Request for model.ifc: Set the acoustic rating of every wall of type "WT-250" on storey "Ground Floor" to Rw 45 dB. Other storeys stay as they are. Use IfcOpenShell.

First a look at what the model holds.

```python
import ifcopenshell
import ifcopenshell.util.element

model = ifcopenshell.open("model.ifc")
print(model.schema)
storey = next(s for s in model.by_type("IfcBuildingStorey") if s.Name == "Ground Floor")
walls = [e for e in ifcopenshell.util.element.get_decomposition(storey) if e.is_a("IfcWall")]
seen = {}
for e in walls:
    element_type = ifcopenshell.util.element.get_type(e)
    key = (element_type.Name if element_type != e and element_type else None, ifcopenshell.util.element.get_pset(e, "Pset_WallCommon", "AcousticRating"))
    seen[key] = seen.get(key, 0) + 1
for (name, value), count in sorted(seen.items(), key=str):
    print(count, "x", name, "|", value)
```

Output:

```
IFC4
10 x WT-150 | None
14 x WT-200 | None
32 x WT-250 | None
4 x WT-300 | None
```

```python
import ifcopenshell
import ifcopenshell.api.pset
import ifcopenshell.util.element

model = ifcopenshell.open("model.ifc")

storey = next(s for s in model.by_type("IfcBuildingStorey") if s.Name == "Ground Floor")
walls = [e for e in ifcopenshell.util.element.get_decomposition(storey) if e.is_a("IfcWall")]

count = 0
for e in walls:
    element_type = ifcopenshell.util.element.get_type(e)
    if element_type in (None, e) or element_type.Name != "WT-250":
        continue
    # add_pset returns the element's existing set when there is one.
    pset = ifcopenshell.api.pset.add_pset(model, product=e, name="Pset_WallCommon")
    ifcopenshell.api.pset.edit_pset(model, pset=pset, properties={"AcousticRating": "Rw 45 dB"})
    count += 1

print(count, "walls updated")

model.write("model_rev.ifc")
```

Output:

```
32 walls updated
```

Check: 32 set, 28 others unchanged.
